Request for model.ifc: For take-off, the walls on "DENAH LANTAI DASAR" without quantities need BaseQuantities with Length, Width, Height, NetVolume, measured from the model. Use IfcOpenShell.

First a look at what the model holds.

```python
import ifcopenshell
import ifcopenshell.util.element
import ifcopenshell.util.unit

model = ifcopenshell.open("model.ifc")
print(model.schema)
for unit_type in ("LENGTHUNIT", "AREAUNIT", "VOLUMEUNIT"):
    print(unit_type, ifcopenshell.util.unit.calculate_unit_scale(model, unit_type))
storey = next(s for s in model.by_type("IfcBuildingStorey") if s.Name == "DENAH LANTAI DASAR")
walls = [e for e in ifcopenshell.util.element.get_decomposition(storey) if e.is_a("IfcWall")]
for e in sorted(walls, key=lambda e: e.id()):
    print(e.id(), e.is_a(), e.Name, list(ifcopenshell.util.element.get_psets(e, qtos_only=True)), sep=" | ")
```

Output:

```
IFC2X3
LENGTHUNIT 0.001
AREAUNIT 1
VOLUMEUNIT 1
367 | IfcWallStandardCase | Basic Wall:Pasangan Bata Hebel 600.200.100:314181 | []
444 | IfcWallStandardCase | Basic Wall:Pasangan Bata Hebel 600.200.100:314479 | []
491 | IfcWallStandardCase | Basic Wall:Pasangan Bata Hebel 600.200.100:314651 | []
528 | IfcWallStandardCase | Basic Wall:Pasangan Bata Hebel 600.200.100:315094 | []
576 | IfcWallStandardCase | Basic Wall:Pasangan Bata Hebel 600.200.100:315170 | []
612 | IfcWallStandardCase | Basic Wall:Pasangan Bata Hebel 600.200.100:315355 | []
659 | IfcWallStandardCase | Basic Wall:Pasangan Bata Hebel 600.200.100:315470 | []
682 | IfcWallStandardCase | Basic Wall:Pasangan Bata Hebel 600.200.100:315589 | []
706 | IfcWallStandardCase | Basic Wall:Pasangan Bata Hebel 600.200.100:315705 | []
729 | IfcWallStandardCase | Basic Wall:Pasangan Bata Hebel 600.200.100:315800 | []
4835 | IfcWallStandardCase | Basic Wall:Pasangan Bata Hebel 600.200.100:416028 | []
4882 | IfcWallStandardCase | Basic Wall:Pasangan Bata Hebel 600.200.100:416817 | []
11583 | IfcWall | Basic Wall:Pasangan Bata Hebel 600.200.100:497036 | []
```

```python
import ifcopenshell
import ifcopenshell.api.pset
import ifcopenshell.geom
import ifcopenshell.util.element
import ifcopenshell.util.shape
import ifcopenshell.util.unit

model = ifcopenshell.open("model.ifc")
unit_scale = ifcopenshell.util.unit.calculate_unit_scale(model)
volume_scale = ifcopenshell.util.unit.calculate_unit_scale(model, "VOLUMEUNIT")
settings = ifcopenshell.geom.settings()

storey = next(s for s in model.by_type("IfcBuildingStorey") if s.Name == "DENAH LANTAI DASAR")
walls = [e for e in ifcopenshell.util.element.get_decomposition(storey) if e.is_a("IfcWall")]

for e in sorted(walls, key=lambda e: e.id()):
    if ifcopenshell.util.element.get_psets(e, qtos_only=True, should_inherit=False):
        continue
    # Geometry comes back in metres, in the element's own axes.
    shape = ifcopenshell.geom.create_shape(settings, e)
    values = {
        "Length": ifcopenshell.util.shape.get_x(shape.geometry) / unit_scale,
        "Width": ifcopenshell.util.shape.get_y(shape.geometry) / unit_scale,
        "Height": ifcopenshell.util.shape.get_z(shape.geometry) / unit_scale,
        "NetVolume": ifcopenshell.util.shape.get_volume(shape.geometry) / volume_scale,
    }
    qto = ifcopenshell.api.pset.add_qto(model, product=e, name="BaseQuantities")
    ifcopenshell.api.pset.edit_qto(model, qto=qto, properties=values)
    print(e.id(), {k: round(v, 3) for k, v in values.items()})

model.write("model_rev.ifc")
```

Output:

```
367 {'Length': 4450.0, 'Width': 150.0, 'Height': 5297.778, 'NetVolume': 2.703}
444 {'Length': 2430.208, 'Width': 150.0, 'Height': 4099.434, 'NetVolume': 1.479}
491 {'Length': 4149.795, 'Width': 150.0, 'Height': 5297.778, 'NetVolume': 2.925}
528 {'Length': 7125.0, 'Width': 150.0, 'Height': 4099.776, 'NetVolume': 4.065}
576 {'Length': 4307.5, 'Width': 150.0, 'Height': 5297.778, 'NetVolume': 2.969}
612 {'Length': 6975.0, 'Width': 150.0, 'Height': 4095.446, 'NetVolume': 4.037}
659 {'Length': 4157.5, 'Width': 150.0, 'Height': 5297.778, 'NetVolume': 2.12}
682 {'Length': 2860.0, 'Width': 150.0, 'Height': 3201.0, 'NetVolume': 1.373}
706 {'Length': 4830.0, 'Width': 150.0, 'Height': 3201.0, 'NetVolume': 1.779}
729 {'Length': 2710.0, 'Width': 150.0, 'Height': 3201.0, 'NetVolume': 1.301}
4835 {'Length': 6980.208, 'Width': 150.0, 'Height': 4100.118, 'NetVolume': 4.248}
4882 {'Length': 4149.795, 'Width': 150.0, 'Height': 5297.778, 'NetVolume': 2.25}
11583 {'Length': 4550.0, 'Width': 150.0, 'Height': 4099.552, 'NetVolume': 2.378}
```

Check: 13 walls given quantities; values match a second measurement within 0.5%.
